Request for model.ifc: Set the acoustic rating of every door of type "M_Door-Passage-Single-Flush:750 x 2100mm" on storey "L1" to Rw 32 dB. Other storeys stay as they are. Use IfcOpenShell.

First a look at what the model holds.

```python
import ifcopenshell
import ifcopenshell.util.element

model = ifcopenshell.open("model.ifc")
print(model.schema)
storey = next(s for s in model.by_type("IfcBuildingStorey") if s.Name == "L1")
doors = [e for e in ifcopenshell.util.element.get_decomposition(storey) if e.is_a("IfcDoor")]
seen = {}
for e in doors:
    element_type = ifcopenshell.util.element.get_type(e)
    key = (element_type.Name if element_type != e and element_type else None, ifcopenshell.util.element.get_pset(e, "Pset_DoorCommon", "AcousticRating"))
    seen[key] = seen.get(key, 0) + 1
for (name, value), count in sorted(seen.items(), key=str):
    print(count, "x", name, "|", value)
```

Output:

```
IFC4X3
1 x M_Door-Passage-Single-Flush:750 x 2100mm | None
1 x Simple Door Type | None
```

```python
import ifcopenshell
import ifcopenshell.api.pset
import ifcopenshell.util.element

model = ifcopenshell.open("model.ifc")

storey = next(s for s in model.by_type("IfcBuildingStorey") if s.Name == "L1")
doors = [e for e in ifcopenshell.util.element.get_decomposition(storey) if e.is_a("IfcDoor")]

count = 0
for e in doors:
    element_type = ifcopenshell.util.element.get_type(e)
    if element_type in (None, e) or element_type.Name != "M_Door-Passage-Single-Flush:750 x 2100mm":
        continue
    # add_pset returns the element's existing set when there is one.
    pset = ifcopenshell.api.pset.add_pset(model, product=e, name="Pset_DoorCommon")
    ifcopenshell.api.pset.edit_pset(model, pset=pset, properties={"AcousticRating": "Rw 32 dB"})
    count += 1

print(count, "doors updated")

model.write("model_rev.ifc")
```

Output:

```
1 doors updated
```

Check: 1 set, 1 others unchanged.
